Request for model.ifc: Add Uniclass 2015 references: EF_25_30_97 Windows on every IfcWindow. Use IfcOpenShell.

First a look at what the model holds.

```python
import ifcopenshell

model = ifcopenshell.open("model.ifc")
print(model.schema)
print("classifications:", [c.Name for c in model.by_type("IfcClassification")])
for ifc_class in ("IfcDoor", "IfcRoof", "IfcStair", "IfcWall", "IfcWindow"):
    print(ifc_class, len(model.by_type(ifc_class)))
```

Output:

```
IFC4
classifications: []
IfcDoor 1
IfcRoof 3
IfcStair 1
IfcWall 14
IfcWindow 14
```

```python
import ifcopenshell
import ifcopenshell.api.classification

model = ifcopenshell.open("model.ifc")

system = ifcopenshell.api.classification.add_classification(model, classification="Uniclass 2015")

codes = {
    "IfcWindow": ("EF_25_30_97", "Windows"),
}
for ifc_class, (code, name) in codes.items():
    products = model.by_type(ifc_class)
    ifcopenshell.api.classification.add_reference(
        model, products=products, classification=system, identification=code, name=name
    )
    print(code, len(products))

model.write("model_edited.ifc")
```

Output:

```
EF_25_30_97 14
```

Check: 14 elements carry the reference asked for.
